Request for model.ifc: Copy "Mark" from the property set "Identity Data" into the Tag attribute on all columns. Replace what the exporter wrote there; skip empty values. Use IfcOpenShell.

First a look at what the model holds.

```python
import ifcopenshell
import ifcopenshell.util.element

model = ifcopenshell.open("model.ifc")
print(model.schema)
columns = model.by_type("IfcColumn")
print(len(columns), "columns")
for e in columns[:8]:
    source = ifcopenshell.util.element.get_pset(e, "Identity Data", "Mark")
    target = e.Tag
    print(e.id(), repr(source), repr(target), sep=" | ")
```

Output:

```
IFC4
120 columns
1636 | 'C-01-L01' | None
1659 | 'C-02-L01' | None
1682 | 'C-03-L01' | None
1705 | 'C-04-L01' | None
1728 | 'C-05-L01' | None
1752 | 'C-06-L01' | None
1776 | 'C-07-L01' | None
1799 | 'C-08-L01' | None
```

```python
import ifcopenshell
import ifcopenshell.util.element

model = ifcopenshell.open("model.ifc")

count = 0
for e in model.by_type("IfcColumn"):
    value = ifcopenshell.util.element.get_pset(e, "Identity Data", "Mark")
    current = e.Tag
    if not value or not value.strip() or current == value:
        continue
    e.Tag = value
    count += 1

print(count, "columns updated")

model.write("model_v2.ifc")
```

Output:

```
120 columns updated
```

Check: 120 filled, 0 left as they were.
